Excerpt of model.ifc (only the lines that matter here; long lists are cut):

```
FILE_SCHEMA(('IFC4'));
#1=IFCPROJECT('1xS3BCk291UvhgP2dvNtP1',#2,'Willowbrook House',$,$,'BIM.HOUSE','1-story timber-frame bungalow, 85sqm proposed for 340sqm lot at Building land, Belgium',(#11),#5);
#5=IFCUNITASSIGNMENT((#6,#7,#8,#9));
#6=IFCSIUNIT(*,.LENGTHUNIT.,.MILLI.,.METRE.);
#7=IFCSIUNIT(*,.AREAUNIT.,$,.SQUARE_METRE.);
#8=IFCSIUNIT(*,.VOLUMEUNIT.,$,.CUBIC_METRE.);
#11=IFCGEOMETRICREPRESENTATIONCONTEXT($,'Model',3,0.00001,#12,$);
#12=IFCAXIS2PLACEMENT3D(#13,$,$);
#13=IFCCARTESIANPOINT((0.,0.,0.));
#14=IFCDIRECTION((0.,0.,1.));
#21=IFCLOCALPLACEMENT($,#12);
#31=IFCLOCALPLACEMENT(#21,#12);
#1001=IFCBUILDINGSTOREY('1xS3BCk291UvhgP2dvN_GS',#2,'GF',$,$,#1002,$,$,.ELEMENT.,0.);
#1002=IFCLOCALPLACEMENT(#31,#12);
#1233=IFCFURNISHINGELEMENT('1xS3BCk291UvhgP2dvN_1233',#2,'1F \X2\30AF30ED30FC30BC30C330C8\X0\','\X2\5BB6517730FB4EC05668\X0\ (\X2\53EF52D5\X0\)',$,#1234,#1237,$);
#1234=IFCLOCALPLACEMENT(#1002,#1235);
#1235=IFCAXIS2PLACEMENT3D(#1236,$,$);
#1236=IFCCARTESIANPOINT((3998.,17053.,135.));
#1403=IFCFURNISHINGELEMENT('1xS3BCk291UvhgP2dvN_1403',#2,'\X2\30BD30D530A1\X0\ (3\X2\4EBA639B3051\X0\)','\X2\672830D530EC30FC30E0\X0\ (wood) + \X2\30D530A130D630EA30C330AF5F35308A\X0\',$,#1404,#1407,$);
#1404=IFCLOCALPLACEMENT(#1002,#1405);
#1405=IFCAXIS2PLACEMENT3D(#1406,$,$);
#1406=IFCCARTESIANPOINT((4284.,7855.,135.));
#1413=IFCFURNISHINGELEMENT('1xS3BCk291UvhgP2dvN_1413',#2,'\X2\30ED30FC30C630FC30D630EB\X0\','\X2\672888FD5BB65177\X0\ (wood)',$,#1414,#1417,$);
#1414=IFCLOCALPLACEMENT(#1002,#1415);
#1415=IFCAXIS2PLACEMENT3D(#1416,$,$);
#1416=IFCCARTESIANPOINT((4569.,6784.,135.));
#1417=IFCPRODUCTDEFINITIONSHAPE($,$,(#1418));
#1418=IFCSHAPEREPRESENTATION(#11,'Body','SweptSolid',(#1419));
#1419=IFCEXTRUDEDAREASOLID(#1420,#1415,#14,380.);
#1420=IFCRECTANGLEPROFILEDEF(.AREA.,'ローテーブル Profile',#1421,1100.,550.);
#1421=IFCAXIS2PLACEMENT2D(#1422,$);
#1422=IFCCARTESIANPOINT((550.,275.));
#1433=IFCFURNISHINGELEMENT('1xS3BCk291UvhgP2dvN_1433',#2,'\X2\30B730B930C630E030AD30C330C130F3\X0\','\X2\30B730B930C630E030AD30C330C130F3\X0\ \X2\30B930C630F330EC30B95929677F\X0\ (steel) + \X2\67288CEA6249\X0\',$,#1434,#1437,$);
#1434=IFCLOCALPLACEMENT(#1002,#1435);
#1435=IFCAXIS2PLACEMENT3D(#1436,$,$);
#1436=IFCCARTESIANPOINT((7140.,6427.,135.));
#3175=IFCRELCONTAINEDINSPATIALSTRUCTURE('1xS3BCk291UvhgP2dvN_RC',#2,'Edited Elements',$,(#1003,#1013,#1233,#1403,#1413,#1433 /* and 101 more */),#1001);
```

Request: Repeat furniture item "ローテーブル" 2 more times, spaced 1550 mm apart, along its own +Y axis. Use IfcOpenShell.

```python
import ifcopenshell
import ifcopenshell.api.geometry
import ifcopenshell.api.root
import ifcopenshell.util.element
import ifcopenshell.util.placement

model = ifcopenshell.open("model.ifc")


def reuse_history(source, copy):
    """copy_class also copies each property set's owner history, people and application; keep the originals."""
    for rel in copy.IsDefinedBy:
        if rel.is_a("IfcRelDefinesByProperties") and (history := rel.RelatingPropertyDefinition.OwnerHistory):
            rel.RelatingPropertyDefinition.OwnerHistory = source.OwnerHistory
            ifcopenshell.util.element.remove_deep2(model, history)


source = model.by_id(1413)
base = ifcopenshell.util.placement.get_local_placement(source.ObjectPlacement)
step = base[:3, 1] * 1550.0

for i in range(1, 3):
    copy = ifcopenshell.api.root.copy_class(model, product=source)
    copy.Representation = ifcopenshell.util.element.copy_deep(
        model, source.Representation, exclude=["IfcGeometricRepresentationContext", "IfcRepresentationMap"]
    )
    reuse_history(source, copy)
    matrix = base.copy()
    matrix[:3, 3] += i * step
    print("added at", matrix[:3, 3].round(3) + 0.0)
    ifcopenshell.api.geometry.edit_object_placement(model, product=copy, matrix=matrix, is_si=False)

model.write("model_rev.ifc")
```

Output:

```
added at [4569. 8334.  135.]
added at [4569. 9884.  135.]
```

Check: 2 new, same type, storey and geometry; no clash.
